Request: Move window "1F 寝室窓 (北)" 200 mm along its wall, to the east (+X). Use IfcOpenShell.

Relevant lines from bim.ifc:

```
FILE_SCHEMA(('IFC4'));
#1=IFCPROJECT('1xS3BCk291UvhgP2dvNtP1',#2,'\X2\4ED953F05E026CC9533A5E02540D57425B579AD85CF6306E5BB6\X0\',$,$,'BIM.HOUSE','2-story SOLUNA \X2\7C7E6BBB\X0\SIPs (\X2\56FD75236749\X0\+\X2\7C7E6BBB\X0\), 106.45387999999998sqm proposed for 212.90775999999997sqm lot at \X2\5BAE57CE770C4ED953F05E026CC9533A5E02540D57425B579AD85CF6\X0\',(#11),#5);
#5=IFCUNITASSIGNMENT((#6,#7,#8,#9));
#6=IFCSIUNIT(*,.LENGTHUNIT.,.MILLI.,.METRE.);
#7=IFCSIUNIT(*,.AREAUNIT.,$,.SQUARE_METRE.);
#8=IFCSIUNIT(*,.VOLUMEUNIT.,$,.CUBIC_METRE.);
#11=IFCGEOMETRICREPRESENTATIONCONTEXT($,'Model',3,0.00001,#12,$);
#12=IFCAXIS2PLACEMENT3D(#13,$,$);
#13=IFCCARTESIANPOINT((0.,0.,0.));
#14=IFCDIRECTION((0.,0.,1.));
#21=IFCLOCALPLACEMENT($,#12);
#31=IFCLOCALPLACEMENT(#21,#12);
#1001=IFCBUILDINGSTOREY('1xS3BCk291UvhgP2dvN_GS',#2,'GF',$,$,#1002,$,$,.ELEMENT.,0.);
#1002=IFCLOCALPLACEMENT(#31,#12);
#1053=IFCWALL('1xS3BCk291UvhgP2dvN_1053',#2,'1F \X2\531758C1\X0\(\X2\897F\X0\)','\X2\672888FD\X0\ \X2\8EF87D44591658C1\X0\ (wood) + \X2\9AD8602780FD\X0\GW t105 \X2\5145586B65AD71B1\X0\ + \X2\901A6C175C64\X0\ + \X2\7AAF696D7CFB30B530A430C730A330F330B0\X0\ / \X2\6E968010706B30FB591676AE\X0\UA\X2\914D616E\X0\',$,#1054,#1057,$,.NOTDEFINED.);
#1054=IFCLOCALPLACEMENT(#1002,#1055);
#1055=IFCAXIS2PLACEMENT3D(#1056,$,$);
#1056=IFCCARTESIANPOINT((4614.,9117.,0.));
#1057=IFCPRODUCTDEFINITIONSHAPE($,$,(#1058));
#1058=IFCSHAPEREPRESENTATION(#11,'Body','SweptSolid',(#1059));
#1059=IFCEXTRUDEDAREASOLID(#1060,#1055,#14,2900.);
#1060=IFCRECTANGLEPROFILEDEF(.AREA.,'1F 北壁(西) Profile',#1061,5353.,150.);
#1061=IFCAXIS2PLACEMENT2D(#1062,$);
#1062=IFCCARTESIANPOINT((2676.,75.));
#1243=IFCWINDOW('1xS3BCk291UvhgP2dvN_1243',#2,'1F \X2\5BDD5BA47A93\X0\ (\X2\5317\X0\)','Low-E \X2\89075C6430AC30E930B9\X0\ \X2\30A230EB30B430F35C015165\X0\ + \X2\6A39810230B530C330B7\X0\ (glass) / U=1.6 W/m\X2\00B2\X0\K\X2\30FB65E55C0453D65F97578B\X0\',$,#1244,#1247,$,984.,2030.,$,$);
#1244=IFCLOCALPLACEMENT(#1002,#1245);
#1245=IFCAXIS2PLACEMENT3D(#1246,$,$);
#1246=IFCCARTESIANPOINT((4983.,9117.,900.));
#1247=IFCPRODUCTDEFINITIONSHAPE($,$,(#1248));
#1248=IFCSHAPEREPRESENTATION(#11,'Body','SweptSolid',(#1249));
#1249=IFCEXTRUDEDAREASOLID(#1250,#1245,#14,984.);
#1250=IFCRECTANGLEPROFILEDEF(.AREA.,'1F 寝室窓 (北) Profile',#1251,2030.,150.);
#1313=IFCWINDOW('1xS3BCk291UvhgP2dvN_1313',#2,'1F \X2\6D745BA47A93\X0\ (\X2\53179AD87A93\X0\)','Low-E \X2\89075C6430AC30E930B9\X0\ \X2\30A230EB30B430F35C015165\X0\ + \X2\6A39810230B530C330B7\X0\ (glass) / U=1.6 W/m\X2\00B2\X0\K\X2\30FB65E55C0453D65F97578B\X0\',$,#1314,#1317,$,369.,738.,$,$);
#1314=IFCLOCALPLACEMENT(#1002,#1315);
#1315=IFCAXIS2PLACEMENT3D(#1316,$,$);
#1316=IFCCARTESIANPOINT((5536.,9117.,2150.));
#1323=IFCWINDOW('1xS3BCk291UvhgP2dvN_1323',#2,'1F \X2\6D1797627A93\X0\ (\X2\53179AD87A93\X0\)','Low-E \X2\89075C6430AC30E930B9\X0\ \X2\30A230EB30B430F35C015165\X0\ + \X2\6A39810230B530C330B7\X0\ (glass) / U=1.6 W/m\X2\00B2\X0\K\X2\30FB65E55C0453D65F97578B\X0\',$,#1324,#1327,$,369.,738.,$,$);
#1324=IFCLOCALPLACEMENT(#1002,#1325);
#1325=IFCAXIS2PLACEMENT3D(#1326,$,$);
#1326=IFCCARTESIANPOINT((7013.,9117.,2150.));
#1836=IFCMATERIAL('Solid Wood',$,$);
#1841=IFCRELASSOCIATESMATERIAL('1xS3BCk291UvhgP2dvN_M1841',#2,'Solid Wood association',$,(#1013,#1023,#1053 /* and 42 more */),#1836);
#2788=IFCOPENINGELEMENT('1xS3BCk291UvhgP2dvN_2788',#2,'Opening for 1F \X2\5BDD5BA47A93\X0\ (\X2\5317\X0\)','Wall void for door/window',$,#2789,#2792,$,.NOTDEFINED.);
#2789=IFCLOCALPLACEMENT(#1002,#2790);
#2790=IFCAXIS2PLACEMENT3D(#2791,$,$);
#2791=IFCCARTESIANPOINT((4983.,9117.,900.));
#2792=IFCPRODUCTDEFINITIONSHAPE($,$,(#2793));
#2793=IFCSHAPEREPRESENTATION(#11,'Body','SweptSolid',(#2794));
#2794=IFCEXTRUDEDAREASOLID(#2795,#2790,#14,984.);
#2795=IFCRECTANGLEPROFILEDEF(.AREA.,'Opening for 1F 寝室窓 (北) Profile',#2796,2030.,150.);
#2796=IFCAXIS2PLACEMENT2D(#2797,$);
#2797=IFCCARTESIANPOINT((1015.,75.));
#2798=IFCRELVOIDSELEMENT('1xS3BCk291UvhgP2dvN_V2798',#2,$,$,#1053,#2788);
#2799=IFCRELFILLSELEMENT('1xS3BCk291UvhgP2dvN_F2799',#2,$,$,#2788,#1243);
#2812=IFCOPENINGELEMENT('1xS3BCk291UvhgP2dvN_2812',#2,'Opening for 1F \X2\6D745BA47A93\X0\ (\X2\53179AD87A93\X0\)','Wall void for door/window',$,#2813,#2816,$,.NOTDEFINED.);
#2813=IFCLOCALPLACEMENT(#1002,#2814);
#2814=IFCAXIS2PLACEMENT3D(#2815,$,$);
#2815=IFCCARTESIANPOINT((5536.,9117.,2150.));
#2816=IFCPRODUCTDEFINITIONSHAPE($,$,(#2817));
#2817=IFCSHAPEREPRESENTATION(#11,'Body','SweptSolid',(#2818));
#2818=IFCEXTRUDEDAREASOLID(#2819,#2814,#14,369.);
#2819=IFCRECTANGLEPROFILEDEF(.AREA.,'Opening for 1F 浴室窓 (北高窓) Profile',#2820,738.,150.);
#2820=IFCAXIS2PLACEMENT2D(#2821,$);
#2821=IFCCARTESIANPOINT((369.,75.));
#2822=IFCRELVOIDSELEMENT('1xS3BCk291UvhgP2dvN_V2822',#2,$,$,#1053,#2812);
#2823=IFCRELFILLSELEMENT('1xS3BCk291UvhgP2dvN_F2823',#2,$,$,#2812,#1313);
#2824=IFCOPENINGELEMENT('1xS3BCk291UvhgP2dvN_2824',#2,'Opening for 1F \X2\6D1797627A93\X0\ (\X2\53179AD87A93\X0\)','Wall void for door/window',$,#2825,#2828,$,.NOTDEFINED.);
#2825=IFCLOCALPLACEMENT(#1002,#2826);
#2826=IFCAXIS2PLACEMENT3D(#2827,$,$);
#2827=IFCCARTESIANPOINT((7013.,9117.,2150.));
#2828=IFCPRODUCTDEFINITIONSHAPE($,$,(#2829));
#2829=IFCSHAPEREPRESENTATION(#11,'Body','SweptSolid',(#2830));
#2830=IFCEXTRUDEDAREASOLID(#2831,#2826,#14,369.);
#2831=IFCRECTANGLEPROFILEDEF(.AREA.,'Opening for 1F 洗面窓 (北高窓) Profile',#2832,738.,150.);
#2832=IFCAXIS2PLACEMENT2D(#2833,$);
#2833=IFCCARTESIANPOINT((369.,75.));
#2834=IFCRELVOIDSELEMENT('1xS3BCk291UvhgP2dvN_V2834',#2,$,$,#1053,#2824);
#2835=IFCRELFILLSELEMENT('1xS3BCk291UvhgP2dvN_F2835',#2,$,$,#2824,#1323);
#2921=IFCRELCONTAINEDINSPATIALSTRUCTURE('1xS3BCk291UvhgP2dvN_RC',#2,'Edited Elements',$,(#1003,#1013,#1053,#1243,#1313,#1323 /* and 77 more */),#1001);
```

```python
import ifcopenshell
import ifcopenshell.api.geometry
import ifcopenshell.util.placement

model = ifcopenshell.open("bim.ifc")

window = model.by_guid("1xS3BCk291UvhgP2dvN_1243")
opening = window.FillsVoids[0].RelatingOpeningElement
wall = opening.VoidsElements[0].RelatingBuildingElement

wall_matrix = ifcopenshell.util.placement.get_local_placement(wall.ObjectPlacement)
shift = wall_matrix[:3, 0] * 200.0
before = ifcopenshell.util.placement.get_local_placement(window.ObjectPlacement)[:3, 3].copy()

# The window is not placed relative to its opening, so move both.
for product in (opening, window):
    matrix = ifcopenshell.util.placement.get_local_placement(product.ObjectPlacement)
    matrix[:3, 3] += shift
    ifcopenshell.api.geometry.edit_object_placement(model, product=product, matrix=matrix, is_si=False)

after = ifcopenshell.util.placement.get_local_placement(window.ObjectPlacement)[:3, 3]
print("window moved by", (after - before).round(3) + 0.0)

model.write("bim_updated.ifc")
```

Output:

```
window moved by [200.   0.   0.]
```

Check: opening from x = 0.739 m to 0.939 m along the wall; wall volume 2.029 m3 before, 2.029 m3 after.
